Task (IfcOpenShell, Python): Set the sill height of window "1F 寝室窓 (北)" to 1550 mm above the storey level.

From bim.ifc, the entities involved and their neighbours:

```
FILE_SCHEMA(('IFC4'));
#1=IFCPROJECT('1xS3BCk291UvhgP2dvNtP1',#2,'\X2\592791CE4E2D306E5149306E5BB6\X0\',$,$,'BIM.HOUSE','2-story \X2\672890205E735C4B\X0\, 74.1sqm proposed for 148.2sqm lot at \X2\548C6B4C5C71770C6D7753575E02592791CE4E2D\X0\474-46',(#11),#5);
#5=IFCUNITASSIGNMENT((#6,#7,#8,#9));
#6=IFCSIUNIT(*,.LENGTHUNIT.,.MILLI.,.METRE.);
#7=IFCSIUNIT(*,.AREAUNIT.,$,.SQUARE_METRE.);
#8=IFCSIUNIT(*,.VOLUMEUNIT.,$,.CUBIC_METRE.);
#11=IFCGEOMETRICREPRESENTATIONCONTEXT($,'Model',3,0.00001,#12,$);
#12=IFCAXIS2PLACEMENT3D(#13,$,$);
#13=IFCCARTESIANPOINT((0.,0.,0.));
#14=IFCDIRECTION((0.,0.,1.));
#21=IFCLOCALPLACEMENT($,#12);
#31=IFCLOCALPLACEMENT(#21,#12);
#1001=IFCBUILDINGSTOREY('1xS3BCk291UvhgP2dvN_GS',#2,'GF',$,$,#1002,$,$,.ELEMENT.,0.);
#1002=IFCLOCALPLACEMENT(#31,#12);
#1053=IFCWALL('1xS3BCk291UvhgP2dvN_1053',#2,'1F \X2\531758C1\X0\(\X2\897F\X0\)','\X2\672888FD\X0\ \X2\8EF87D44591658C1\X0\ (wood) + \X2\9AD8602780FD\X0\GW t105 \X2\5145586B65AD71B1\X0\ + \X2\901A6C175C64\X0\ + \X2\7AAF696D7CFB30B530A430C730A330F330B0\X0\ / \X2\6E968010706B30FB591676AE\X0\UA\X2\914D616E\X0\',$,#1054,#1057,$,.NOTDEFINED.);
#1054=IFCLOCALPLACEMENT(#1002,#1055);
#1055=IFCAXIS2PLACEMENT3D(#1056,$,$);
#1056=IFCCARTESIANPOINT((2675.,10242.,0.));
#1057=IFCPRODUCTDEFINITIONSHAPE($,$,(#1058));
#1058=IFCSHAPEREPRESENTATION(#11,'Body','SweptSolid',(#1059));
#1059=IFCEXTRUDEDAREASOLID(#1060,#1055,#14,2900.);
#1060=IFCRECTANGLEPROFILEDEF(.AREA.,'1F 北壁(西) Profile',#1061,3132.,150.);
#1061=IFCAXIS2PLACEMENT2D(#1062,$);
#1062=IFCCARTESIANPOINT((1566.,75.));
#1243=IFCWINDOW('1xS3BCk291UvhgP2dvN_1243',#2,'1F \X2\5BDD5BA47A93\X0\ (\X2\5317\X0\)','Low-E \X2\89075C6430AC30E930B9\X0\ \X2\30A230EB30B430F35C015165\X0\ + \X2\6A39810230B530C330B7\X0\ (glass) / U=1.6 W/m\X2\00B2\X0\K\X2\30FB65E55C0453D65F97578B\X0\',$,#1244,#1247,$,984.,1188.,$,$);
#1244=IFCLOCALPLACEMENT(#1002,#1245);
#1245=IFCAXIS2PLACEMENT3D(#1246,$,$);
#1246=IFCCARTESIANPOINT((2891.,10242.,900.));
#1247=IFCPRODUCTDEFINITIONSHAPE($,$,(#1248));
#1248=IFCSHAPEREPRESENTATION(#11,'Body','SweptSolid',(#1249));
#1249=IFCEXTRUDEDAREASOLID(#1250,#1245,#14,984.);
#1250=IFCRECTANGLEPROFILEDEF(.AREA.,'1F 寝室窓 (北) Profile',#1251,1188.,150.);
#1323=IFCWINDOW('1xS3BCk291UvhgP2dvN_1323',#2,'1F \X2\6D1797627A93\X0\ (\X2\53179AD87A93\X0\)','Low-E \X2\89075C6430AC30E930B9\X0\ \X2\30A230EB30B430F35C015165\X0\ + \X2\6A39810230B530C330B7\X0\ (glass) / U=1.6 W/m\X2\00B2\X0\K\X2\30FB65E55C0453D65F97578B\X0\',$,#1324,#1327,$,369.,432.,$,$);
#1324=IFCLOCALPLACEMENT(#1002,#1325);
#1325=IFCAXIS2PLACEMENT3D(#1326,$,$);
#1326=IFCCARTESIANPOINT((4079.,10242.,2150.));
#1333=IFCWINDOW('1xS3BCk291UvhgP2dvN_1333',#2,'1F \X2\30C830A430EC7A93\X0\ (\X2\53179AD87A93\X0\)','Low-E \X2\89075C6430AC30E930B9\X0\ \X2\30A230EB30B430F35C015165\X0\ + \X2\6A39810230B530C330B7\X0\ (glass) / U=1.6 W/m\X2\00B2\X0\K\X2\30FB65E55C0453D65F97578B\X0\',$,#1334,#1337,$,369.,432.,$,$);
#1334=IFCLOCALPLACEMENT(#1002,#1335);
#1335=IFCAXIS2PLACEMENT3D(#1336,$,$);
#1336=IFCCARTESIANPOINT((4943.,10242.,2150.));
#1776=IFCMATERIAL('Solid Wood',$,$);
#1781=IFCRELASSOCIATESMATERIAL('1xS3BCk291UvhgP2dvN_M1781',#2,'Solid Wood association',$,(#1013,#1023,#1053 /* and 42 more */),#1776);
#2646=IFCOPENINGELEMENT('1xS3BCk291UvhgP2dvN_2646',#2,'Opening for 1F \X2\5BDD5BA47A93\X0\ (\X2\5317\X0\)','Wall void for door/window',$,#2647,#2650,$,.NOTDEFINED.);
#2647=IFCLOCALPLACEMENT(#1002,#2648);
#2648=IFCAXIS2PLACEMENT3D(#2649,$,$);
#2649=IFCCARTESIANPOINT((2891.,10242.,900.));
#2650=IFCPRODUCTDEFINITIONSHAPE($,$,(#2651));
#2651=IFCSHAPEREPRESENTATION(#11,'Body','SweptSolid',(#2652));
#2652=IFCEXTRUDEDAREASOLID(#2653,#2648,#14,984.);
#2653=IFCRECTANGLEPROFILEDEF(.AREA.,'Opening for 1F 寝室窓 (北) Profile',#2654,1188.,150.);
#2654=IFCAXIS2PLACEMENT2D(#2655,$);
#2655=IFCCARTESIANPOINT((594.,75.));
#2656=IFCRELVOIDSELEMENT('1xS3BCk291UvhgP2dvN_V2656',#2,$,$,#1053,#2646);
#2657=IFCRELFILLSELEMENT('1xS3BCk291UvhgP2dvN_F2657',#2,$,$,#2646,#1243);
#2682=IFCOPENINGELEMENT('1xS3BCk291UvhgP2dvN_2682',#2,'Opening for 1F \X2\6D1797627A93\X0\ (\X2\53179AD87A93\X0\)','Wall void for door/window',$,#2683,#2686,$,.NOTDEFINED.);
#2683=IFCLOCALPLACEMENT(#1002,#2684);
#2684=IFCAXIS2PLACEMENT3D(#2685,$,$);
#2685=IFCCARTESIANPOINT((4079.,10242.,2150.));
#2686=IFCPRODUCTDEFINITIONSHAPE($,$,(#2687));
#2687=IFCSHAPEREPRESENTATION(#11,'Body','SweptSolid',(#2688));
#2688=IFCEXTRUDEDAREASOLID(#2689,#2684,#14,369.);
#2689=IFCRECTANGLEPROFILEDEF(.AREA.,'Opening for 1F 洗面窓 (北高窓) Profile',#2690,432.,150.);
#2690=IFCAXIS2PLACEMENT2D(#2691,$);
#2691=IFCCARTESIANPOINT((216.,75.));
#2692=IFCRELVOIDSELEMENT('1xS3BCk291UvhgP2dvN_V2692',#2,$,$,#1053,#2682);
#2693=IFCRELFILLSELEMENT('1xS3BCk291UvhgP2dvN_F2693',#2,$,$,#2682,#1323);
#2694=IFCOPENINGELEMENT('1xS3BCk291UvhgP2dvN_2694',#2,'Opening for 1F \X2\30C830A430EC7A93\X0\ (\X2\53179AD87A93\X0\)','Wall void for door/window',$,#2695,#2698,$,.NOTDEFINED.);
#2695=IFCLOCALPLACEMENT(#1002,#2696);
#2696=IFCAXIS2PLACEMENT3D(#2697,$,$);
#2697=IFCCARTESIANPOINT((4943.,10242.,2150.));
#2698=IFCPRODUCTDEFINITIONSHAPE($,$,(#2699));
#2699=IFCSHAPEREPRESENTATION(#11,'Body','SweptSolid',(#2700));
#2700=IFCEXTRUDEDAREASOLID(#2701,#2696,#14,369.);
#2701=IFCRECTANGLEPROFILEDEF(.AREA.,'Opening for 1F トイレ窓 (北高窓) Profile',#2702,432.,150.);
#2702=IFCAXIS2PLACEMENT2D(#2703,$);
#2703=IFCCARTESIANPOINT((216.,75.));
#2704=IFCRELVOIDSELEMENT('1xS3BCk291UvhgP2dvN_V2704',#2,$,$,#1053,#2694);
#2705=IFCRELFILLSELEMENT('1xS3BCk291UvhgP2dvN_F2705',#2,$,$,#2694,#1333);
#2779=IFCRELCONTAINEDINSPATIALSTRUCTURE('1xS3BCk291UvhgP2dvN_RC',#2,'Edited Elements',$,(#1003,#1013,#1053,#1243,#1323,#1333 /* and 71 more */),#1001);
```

```python
import numpy as np
import ifcopenshell
import ifcopenshell.api.geometry
import ifcopenshell.geom
import ifcopenshell.util.element
import ifcopenshell.util.placement
import ifcopenshell.util.shape
import ifcopenshell.util.unit

model = ifcopenshell.open("bim.ifc")
unit_scale = ifcopenshell.util.unit.calculate_unit_scale(model)

window = model.by_guid("1xS3BCk291UvhgP2dvN_1243")
opening = window.FillsVoids[0].RelatingOpeningElement
storey = ifcopenshell.util.element.get_container(window, ifc_class="IfcBuildingStorey")
level = ifcopenshell.util.placement.get_local_placement(storey.ObjectPlacement)[2, 3]

# The opening's origin need not be at the sill, so measure its lowest point.
shape = ifcopenshell.geom.create_shape(ifcopenshell.geom.settings(), opening)
bottom = ifcopenshell.util.shape.get_shape_bottom_elevation(shape, shape.geometry) / unit_scale
dz = level + 1550.0 - bottom

shift = np.array([0.0, 0.0, dz])
# The window is not placed relative to its opening, so move both.
for product in (opening, window):
    matrix = ifcopenshell.util.placement.get_local_placement(product.ObjectPlacement)
    matrix[:3, 3] += shift
    ifcopenshell.api.geometry.edit_object_placement(model, product=product, matrix=matrix, is_si=False)

print(f"moved by {dz * unit_scale:+.3f} m")

model.write("bim_updated.ifc")
```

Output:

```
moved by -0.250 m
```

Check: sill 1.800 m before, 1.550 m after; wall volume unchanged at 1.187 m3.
